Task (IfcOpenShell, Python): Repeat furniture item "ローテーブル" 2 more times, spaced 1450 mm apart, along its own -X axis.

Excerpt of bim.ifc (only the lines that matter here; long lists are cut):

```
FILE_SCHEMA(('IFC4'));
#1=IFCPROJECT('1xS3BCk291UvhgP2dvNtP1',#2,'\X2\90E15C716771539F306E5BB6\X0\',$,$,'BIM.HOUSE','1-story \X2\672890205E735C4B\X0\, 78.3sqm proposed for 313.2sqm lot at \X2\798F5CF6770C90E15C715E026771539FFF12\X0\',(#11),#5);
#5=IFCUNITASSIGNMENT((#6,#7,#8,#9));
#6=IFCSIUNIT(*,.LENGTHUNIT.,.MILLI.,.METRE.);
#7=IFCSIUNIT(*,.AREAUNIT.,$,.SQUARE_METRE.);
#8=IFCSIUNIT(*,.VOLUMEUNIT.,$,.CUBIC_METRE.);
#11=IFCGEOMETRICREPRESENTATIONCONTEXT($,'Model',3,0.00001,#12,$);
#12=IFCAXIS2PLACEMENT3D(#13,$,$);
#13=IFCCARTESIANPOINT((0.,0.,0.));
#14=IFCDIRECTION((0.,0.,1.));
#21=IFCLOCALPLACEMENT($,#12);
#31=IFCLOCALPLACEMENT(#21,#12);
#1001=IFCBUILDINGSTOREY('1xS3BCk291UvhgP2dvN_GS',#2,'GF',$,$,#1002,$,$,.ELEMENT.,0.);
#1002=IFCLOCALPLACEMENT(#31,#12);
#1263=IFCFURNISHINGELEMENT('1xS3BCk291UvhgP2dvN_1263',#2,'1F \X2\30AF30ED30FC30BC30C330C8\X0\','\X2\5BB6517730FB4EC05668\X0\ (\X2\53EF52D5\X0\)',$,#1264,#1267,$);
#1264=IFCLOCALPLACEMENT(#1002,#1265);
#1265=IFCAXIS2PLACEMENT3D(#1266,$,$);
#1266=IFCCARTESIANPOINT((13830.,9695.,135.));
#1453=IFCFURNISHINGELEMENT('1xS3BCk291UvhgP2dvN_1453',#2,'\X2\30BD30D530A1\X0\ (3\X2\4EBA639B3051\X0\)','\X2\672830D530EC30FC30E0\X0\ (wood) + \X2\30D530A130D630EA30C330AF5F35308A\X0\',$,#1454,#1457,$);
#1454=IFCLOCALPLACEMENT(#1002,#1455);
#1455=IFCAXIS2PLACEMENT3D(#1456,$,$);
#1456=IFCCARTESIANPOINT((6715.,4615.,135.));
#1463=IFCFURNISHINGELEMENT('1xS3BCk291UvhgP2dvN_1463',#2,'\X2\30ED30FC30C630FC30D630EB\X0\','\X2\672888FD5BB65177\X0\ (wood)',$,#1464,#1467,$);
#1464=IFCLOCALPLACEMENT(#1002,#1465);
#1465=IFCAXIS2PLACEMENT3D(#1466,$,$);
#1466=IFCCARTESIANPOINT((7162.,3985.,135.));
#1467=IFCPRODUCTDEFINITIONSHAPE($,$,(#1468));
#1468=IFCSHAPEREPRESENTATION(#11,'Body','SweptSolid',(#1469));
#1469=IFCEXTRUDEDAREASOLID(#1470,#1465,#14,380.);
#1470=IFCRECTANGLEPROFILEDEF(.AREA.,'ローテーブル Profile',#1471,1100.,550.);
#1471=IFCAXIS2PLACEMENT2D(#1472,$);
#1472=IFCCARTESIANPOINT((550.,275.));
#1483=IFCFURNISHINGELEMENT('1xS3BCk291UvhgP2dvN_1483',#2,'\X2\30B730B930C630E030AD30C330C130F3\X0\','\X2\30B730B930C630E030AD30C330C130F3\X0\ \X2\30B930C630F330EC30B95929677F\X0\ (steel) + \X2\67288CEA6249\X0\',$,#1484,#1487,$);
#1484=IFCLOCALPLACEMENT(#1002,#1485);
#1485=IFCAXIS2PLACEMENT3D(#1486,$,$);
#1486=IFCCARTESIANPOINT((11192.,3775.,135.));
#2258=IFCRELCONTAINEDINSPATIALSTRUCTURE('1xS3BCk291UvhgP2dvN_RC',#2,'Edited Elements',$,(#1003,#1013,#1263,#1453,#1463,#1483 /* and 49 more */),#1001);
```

```python
import ifcopenshell
import ifcopenshell.api.geometry
import ifcopenshell.api.root
import ifcopenshell.util.element
import ifcopenshell.util.placement
import ifcopenshell.util.unit

model = ifcopenshell.open("bim.ifc")
unit_scale = ifcopenshell.util.unit.calculate_unit_scale(model)


def reuse_history(source, copy):
    """copy_class also copies each property set's owner history, people and application; keep the originals."""
    for rel in copy.IsDefinedBy:
        if rel.is_a("IfcRelDefinesByProperties") and (history := rel.RelatingPropertyDefinition.OwnerHistory):
            rel.RelatingPropertyDefinition.OwnerHistory = source.OwnerHistory
            ifcopenshell.util.element.remove_deep2(model, history)


source = model.by_guid("1xS3BCk291UvhgP2dvN_1463")
base = ifcopenshell.util.placement.get_local_placement(source.ObjectPlacement)
step = -base[:3, 0] * 1.45 / unit_scale

for i in range(1, 3):
    copy = ifcopenshell.api.root.copy_class(model, product=source)
    copy.Representation = ifcopenshell.util.element.copy_deep(
        model, source.Representation, exclude=["IfcGeometricRepresentationContext", "IfcRepresentationMap"]
    )
    reuse_history(source, copy)
    matrix = base.copy()
    matrix[:3, 3] += i * step
    print("added at", matrix[:3, 3].round(3) + 0.0)
    ifcopenshell.api.geometry.edit_object_placement(model, product=copy, matrix=matrix, is_si=False)

model.write("bim_edited.ifc")
```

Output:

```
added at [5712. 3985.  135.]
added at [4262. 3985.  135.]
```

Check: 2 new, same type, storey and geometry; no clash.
